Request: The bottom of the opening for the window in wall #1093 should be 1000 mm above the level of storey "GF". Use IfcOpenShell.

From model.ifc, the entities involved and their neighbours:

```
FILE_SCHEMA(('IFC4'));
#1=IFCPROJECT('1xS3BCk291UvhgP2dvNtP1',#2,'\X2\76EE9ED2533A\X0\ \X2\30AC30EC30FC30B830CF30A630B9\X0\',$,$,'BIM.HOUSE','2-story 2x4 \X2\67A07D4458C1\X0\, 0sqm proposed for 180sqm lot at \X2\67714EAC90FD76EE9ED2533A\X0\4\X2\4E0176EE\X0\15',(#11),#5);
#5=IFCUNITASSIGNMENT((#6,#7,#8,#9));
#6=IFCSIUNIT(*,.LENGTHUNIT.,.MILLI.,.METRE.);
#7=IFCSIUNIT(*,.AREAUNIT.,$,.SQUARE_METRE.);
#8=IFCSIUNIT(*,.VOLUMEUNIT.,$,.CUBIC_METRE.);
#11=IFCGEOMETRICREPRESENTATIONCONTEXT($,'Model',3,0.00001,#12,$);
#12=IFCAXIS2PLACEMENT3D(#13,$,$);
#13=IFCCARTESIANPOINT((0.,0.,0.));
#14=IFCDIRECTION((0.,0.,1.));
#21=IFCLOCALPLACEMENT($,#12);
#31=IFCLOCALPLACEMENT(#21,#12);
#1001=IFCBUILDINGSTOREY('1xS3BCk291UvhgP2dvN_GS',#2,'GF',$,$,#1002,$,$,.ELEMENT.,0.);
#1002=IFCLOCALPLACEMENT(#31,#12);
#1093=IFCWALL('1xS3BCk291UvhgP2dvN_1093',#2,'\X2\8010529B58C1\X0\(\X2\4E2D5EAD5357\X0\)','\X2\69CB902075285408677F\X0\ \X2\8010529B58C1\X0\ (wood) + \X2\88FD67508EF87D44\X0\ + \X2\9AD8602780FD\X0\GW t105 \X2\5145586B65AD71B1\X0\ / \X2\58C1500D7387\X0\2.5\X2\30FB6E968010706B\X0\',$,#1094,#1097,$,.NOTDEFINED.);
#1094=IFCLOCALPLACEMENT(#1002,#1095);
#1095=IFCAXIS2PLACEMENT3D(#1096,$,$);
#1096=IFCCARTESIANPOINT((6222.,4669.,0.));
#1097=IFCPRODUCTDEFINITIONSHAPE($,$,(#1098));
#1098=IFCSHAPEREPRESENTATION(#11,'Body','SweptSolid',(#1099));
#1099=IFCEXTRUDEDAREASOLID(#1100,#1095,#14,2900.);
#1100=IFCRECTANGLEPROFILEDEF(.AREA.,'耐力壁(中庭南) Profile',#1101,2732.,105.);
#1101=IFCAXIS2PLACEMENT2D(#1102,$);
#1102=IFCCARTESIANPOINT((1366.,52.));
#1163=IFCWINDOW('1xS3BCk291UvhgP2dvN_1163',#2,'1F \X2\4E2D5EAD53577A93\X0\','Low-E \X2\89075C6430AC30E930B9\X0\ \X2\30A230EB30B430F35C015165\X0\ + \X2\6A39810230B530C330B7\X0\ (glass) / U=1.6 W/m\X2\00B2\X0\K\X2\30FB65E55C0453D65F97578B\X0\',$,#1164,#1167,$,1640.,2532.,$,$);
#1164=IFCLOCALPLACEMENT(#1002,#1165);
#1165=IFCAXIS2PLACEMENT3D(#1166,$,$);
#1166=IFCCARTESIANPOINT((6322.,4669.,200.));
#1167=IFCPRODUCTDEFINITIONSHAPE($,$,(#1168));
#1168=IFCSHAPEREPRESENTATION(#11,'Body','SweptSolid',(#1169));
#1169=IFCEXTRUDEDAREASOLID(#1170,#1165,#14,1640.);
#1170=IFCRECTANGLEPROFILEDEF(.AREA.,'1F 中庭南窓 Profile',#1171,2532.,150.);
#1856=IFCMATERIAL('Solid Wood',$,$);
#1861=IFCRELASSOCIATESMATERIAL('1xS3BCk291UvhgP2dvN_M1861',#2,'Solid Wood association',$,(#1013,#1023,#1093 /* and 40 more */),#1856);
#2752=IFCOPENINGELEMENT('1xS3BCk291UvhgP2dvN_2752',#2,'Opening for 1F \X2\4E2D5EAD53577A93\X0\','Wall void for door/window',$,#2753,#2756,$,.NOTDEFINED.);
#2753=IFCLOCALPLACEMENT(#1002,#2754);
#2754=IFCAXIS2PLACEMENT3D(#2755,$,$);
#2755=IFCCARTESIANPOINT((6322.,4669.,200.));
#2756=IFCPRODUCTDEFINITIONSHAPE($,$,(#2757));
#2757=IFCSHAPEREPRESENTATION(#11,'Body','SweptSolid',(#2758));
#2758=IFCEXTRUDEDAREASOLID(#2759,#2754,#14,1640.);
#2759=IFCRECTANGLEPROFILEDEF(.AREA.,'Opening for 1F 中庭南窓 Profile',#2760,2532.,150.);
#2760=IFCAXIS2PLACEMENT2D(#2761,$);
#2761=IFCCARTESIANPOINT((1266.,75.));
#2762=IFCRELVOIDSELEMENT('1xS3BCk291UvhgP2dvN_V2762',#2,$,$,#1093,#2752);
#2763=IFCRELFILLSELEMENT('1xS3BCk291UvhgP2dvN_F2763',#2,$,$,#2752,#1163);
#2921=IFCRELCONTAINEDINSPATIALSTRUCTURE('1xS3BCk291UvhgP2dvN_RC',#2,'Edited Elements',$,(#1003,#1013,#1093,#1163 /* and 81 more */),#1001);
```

```python
import numpy as np
import ifcopenshell
import ifcopenshell.api.geometry
import ifcopenshell.geom
import ifcopenshell.util.element
import ifcopenshell.util.placement
import ifcopenshell.util.shape
import ifcopenshell.util.unit

model = ifcopenshell.open("model.ifc")
unit_scale = ifcopenshell.util.unit.calculate_unit_scale(model)

window = model.by_guid("1xS3BCk291UvhgP2dvN_1163")
opening = window.FillsVoids[0].RelatingOpeningElement
storey = ifcopenshell.util.element.get_container(window, ifc_class="IfcBuildingStorey")
level = ifcopenshell.util.placement.get_local_placement(storey.ObjectPlacement)[2, 3]

# The opening's origin need not be at the sill, so measure its lowest point.
shape = ifcopenshell.geom.create_shape(ifcopenshell.geom.settings(), opening)
bottom = ifcopenshell.util.shape.get_shape_bottom_elevation(shape, shape.geometry) / unit_scale
dz = level + 1000.0 - bottom

shift = np.array([0.0, 0.0, dz])
# The window is not placed relative to its opening, so move both.
for product in (opening, window):
    matrix = ifcopenshell.util.placement.get_local_placement(product.ObjectPlacement)
    matrix[:3, 3] += shift
    ifcopenshell.api.geometry.edit_object_placement(model, product=product, matrix=matrix, is_si=False)

print(f"moved by {dz * unit_scale:+.3f} m")

model.write("model_v2.ifc")
```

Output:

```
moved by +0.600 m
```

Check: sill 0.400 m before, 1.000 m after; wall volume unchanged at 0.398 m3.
